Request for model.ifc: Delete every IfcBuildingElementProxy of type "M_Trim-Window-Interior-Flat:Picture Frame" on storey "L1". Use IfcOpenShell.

First a look at what the model holds.

```python
import ifcopenshell
import ifcopenshell.util.element

model = ifcopenshell.open("model.ifc")
print(model.schema)
storey = next(s for s in model.by_type("IfcBuildingStorey") if s.Name == "L1")
proxies = [e for e in ifcopenshell.util.element.get_decomposition(storey) if e.is_a("IfcBuildingElementProxy")]
seen = {}
for e in proxies:
    element_type = ifcopenshell.util.element.get_type(e)
    name = element_type.Name if element_type not in (None, e) else None
    seen[name] = seen.get(name, 0) + 1
for name, count in sorted(seen.items(), key=str):
    print(count, "x", name)
```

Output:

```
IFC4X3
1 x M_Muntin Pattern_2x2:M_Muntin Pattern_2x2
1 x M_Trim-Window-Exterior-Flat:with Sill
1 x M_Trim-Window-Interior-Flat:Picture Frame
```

```python
import ifcopenshell
import ifcopenshell.api.root
import ifcopenshell.util.element

model = ifcopenshell.open("model.ifc")

storey = next(s for s in model.by_type("IfcBuildingStorey") if s.Name == "L1")
proxies = [e for e in ifcopenshell.util.element.get_decomposition(storey) if e.is_a("IfcBuildingElementProxy")]
targets = [e for e in proxies if (t := ifcopenshell.util.element.get_type(e)) not in (None, e) and t.Name == "M_Trim-Window-Interior-Flat:Picture Frame"]

for e in targets:
    ifcopenshell.api.root.remove_product(model, product=e)
print(len(targets), "removed")

model.write("model_updated.ifc")
```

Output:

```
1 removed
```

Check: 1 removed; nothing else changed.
